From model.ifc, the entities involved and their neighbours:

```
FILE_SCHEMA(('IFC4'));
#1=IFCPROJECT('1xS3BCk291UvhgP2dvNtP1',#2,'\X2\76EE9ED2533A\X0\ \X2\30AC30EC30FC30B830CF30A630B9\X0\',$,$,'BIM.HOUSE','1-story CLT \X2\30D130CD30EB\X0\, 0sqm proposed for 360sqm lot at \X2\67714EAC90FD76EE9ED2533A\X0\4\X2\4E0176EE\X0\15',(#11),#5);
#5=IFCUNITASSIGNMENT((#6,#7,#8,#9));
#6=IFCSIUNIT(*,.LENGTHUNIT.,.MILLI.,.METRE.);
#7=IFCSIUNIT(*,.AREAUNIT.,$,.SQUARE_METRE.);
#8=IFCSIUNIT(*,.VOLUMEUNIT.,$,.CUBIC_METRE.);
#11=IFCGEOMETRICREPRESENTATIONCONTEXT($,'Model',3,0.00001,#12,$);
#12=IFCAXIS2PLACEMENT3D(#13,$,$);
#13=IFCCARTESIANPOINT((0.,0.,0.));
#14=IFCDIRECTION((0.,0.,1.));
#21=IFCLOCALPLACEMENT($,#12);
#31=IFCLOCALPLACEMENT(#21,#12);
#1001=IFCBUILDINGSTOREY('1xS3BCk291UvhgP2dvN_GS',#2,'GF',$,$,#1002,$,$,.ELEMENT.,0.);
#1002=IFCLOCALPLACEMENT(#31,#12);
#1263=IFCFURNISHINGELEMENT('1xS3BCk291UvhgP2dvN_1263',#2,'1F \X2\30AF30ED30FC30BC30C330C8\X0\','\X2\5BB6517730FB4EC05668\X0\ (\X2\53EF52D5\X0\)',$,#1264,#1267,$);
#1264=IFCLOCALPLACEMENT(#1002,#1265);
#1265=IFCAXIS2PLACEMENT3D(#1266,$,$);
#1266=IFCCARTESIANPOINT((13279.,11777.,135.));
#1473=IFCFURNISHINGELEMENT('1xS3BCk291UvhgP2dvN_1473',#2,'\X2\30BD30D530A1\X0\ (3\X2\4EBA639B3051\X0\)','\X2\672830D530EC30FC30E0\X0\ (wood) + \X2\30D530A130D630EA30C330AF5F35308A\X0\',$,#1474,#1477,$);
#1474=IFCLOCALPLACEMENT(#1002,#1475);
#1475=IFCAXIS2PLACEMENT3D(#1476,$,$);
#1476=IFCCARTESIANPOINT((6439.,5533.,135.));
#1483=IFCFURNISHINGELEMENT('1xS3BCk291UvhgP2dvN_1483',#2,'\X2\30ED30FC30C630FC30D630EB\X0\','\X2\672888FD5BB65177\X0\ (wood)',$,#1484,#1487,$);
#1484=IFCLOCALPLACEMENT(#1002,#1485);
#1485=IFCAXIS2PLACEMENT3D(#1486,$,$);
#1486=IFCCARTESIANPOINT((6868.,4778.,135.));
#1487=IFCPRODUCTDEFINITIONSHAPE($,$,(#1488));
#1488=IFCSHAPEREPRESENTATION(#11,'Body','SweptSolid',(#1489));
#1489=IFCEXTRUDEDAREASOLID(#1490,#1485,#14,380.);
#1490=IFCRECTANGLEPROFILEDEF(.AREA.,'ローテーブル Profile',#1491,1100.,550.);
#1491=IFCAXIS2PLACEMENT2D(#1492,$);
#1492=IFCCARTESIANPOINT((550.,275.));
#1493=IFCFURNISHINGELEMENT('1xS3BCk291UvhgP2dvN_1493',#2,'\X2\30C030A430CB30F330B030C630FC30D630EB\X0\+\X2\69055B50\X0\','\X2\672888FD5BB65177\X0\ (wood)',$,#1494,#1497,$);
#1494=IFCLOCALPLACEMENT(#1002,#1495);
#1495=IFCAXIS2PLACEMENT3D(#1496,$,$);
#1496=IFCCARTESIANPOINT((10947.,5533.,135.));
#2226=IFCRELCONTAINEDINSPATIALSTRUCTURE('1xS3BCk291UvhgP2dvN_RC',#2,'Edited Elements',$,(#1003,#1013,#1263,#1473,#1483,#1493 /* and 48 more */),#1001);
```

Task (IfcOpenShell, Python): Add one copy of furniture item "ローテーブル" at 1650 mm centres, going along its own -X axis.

```python
import ifcopenshell
import ifcopenshell.api.geometry
import ifcopenshell.api.root
import ifcopenshell.util.element
import ifcopenshell.util.placement
import ifcopenshell.util.unit

model = ifcopenshell.open("model.ifc")
unit_scale = ifcopenshell.util.unit.calculate_unit_scale(model)


def reuse_history(source, copy):
    """copy_class also copies each property set's owner history, people and application; keep the originals."""
    for rel in copy.IsDefinedBy:
        if rel.is_a("IfcRelDefinesByProperties") and (history := rel.RelatingPropertyDefinition.OwnerHistory):
            rel.RelatingPropertyDefinition.OwnerHistory = source.OwnerHistory
            ifcopenshell.util.element.remove_deep2(model, history)


source = model.by_guid("1xS3BCk291UvhgP2dvN_1483")
base = ifcopenshell.util.placement.get_local_placement(source.ObjectPlacement)
step = -base[:3, 0] * 1.65 / unit_scale

for i in range(1, 2):
    copy = ifcopenshell.api.root.copy_class(model, product=source)
    copy.Representation = ifcopenshell.util.element.copy_deep(
        model, source.Representation, exclude=["IfcGeometricRepresentationContext", "IfcRepresentationMap"]
    )
    reuse_history(source, copy)
    matrix = base.copy()
    matrix[:3, 3] += i * step
    print("added at", matrix[:3, 3].round(3) + 0.0)
    ifcopenshell.api.geometry.edit_object_placement(model, product=copy, matrix=matrix, is_si=False)

model.write("model_edited.ifc")
```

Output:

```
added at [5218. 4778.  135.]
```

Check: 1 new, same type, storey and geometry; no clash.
